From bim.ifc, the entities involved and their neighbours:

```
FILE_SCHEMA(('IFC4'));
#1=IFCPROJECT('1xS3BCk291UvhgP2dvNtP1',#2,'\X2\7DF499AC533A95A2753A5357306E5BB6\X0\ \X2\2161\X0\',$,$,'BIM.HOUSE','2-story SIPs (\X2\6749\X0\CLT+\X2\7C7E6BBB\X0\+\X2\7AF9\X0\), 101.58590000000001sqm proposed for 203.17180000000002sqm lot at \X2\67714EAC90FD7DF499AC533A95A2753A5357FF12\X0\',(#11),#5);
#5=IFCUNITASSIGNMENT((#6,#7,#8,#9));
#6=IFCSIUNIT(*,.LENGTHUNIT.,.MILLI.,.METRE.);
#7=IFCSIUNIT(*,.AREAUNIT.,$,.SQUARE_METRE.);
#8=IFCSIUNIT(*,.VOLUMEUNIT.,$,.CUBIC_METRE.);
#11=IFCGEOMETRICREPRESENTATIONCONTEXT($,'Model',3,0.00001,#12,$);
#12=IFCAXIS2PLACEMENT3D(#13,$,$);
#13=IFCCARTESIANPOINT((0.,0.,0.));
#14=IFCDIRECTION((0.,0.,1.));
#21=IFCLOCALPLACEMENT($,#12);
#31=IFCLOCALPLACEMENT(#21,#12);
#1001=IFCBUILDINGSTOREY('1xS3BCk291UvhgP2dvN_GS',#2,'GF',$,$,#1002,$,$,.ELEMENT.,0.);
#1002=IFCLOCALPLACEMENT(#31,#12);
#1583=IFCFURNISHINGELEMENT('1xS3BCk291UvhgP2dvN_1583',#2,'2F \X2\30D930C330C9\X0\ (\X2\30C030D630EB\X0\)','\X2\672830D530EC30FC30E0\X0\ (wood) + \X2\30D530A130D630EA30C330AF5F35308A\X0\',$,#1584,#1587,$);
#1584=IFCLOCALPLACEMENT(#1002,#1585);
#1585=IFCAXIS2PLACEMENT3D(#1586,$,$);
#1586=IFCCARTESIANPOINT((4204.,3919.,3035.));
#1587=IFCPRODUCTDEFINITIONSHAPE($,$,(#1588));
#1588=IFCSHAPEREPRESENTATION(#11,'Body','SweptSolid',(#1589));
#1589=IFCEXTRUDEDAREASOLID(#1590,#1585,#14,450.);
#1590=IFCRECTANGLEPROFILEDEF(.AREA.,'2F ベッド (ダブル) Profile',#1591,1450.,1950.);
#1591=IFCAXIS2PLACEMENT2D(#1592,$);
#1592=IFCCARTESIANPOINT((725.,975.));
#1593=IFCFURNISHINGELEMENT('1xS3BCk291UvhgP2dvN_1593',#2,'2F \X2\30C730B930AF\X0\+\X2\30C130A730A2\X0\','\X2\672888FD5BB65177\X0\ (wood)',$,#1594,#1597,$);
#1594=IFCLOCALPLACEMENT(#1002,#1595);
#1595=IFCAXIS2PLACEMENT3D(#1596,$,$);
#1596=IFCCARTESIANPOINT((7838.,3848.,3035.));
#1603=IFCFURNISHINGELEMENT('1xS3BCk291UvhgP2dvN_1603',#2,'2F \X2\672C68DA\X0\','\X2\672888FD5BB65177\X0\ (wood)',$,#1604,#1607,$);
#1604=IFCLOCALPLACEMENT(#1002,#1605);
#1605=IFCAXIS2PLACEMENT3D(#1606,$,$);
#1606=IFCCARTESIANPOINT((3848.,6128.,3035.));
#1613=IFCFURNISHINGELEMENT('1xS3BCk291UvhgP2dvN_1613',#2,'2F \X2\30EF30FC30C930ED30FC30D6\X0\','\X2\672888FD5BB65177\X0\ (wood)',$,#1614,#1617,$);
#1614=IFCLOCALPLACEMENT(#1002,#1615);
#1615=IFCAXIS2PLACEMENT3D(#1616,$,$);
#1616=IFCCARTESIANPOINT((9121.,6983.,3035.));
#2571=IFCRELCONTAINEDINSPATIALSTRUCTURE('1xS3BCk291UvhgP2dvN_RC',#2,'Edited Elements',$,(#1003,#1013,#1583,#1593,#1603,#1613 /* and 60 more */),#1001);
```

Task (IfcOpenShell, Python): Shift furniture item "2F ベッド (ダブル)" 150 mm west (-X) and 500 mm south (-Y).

```python
import ifcopenshell
import ifcopenshell.api.geometry
import ifcopenshell.util.placement
import ifcopenshell.util.unit

model = ifcopenshell.open("bim.ifc")
unit_scale = ifcopenshell.util.unit.calculate_unit_scale(model)

item = model.by_guid("1xS3BCk291UvhgP2dvN_1583")
matrix = ifcopenshell.util.placement.get_local_placement(item.ObjectPlacement)
matrix[0, 3] -= 0.15 / unit_scale
matrix[1, 3] -= 0.5 / unit_scale
ifcopenshell.api.geometry.edit_object_placement(model, product=item, matrix=matrix, is_si=False)

print(ifcopenshell.util.placement.get_local_placement(item.ObjectPlacement).round(3) + 0.0)

model.write("bim-out.ifc")
```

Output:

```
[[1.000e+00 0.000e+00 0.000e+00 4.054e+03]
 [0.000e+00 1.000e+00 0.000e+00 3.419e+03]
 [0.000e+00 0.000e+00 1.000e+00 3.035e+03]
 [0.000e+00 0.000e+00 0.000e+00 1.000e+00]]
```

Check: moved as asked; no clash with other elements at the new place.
